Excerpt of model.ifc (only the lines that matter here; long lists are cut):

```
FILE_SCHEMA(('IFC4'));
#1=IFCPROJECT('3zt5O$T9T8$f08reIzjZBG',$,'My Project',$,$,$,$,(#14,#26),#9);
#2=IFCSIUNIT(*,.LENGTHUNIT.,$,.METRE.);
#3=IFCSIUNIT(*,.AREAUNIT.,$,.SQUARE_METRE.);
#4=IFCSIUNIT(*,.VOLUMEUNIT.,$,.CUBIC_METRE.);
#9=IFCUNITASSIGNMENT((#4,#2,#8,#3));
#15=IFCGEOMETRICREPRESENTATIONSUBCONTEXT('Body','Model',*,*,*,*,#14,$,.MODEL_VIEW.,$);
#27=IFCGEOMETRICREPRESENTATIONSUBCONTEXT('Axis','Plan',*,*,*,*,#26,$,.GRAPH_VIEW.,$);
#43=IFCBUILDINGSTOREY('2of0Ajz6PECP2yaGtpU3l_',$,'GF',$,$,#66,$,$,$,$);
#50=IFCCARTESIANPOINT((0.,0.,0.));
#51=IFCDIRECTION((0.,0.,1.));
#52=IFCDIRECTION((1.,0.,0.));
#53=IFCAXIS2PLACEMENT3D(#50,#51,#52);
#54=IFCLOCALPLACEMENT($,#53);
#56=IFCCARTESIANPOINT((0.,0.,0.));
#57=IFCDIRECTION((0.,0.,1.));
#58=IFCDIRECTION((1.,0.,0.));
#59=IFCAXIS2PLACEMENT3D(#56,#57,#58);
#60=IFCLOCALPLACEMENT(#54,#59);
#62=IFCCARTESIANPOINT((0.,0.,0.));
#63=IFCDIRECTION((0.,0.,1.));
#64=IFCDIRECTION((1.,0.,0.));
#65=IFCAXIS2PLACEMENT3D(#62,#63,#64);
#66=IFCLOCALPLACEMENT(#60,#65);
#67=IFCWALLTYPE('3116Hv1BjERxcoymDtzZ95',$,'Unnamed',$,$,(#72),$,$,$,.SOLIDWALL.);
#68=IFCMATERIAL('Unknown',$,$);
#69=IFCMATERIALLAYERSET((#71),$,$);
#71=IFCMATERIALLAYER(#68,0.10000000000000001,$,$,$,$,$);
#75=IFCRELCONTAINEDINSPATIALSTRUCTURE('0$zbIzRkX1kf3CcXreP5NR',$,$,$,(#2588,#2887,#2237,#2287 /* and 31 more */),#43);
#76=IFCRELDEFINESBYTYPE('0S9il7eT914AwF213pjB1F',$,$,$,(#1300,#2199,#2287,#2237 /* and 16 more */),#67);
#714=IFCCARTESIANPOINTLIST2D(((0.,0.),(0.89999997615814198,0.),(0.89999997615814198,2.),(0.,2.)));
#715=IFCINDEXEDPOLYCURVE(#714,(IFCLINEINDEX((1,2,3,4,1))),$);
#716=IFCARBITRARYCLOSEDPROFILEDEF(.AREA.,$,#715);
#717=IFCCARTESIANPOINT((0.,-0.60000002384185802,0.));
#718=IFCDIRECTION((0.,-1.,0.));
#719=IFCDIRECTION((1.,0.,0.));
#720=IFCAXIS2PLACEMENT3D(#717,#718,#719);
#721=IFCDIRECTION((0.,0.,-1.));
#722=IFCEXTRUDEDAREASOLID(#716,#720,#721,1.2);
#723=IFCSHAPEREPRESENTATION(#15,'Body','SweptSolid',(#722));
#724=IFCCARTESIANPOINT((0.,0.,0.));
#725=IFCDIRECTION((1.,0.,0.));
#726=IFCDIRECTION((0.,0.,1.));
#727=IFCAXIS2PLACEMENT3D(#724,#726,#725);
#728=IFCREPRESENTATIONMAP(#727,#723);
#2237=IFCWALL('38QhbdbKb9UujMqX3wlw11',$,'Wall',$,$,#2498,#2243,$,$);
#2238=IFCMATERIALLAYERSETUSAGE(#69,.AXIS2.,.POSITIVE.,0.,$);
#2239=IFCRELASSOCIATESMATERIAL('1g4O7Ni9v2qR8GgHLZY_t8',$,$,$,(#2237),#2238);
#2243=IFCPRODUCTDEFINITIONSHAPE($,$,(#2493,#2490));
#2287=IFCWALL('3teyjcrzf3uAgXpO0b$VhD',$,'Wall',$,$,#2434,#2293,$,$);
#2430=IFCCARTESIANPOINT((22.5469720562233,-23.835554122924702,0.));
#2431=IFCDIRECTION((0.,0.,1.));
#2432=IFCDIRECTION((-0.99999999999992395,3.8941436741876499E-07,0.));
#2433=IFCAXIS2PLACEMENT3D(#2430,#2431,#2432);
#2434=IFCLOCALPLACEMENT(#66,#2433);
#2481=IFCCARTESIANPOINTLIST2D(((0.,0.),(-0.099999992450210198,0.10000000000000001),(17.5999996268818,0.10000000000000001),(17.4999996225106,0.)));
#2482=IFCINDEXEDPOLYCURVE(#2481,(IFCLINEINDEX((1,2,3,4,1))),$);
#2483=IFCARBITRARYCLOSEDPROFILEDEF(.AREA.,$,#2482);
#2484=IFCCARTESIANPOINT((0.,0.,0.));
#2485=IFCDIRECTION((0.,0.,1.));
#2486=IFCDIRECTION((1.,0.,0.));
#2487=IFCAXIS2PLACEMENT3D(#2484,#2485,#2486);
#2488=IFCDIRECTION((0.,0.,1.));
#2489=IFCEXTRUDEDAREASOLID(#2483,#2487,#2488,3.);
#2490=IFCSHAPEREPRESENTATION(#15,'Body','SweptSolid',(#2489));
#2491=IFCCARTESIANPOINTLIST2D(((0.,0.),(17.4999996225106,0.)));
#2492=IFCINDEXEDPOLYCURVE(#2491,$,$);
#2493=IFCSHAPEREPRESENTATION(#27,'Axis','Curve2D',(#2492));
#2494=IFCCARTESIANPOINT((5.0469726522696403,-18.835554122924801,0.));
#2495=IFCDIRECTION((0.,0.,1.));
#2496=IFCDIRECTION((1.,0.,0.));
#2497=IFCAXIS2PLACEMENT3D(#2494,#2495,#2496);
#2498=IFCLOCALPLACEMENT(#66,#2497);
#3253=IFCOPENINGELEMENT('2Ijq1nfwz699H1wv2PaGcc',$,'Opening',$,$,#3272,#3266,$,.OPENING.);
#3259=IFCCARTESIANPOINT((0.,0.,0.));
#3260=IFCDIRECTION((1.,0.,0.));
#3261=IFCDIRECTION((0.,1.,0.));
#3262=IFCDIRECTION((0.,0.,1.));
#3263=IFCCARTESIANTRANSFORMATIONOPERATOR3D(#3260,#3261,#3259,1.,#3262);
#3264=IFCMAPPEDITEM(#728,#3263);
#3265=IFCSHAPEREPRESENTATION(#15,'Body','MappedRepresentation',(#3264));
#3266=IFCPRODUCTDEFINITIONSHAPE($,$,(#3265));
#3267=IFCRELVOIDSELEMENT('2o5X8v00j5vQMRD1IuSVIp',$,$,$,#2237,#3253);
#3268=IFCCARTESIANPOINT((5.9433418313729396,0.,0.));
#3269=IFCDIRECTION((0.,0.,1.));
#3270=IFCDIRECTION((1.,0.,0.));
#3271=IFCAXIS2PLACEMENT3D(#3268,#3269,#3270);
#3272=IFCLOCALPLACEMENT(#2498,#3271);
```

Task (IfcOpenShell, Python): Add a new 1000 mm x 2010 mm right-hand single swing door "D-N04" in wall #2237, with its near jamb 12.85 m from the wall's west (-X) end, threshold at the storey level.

```python
import numpy as np
import ifcopenshell
import ifcopenshell.api.feature
import ifcopenshell.api.geometry
import ifcopenshell.api.root
import ifcopenshell.api.spatial
import ifcopenshell.geom
import ifcopenshell.util.element
import ifcopenshell.util.placement
import ifcopenshell.util.representation
import ifcopenshell.util.shape
import ifcopenshell.util.unit

model = ifcopenshell.open("model.ifc")
unit_scale = ifcopenshell.util.unit.calculate_unit_scale(model)
settings = ifcopenshell.geom.settings()


def volume(element):
    """Net volume in cubic metres, openings subtracted."""
    shape = ifcopenshell.geom.create_shape(settings, element)
    return ifcopenshell.util.shape.get_volume(shape.geometry)


wall = model.by_id(2237)
storey = ifcopenshell.util.element.get_container(wall, ifc_class="IfcBuildingStorey")
context = ifcopenshell.util.representation.get_context(model, "Model", "Body", "MODEL_VIEW")
before = volume(wall)

width, height, from_end, sill = 1, 2.01, 12.85, 0.0  # metres

# The wall runs along its own X axis, and the end named is its -X end.
wall_shape = ifcopenshell.geom.create_shape(settings, wall)
x, y, z = ifcopenshell.util.shape.get_vertices(wall_shape.geometry).T
start = x.min() + from_end
face, thickness = float(y.min()), float(y.max() - y.min())
wall_matrix = ifcopenshell.util.placement.get_local_placement(wall.ObjectPlacement)
level = ifcopenshell.util.placement.get_local_placement(storey.ObjectPlacement)[2, 3]


def in_wall(x, y):
    """Placement at x, y metres in the wall's axes, at sill height."""
    matrix = wall_matrix.copy()
    matrix[:, 3] = wall_matrix @ np.array([x / unit_scale, y / unit_scale, 0.0, 1.0])
    matrix[2, 3] = level + sill / unit_scale
    return matrix


# Opening: a box that overshoots both wall faces by 50 mm.
opening = ifcopenshell.api.root.create_entity(model, ifc_class="IfcOpeningElement", predefined_type="OPENING")
box = ifcopenshell.api.geometry.add_wall_representation(
    model, context=context, length=width, height=height, thickness=thickness + 0.1
)
ifcopenshell.api.geometry.assign_representation(model, product=opening, representation=box)
ifcopenshell.api.geometry.edit_object_placement(model, product=opening, matrix=in_wall(start, face - 0.05), is_si=False)
ifcopenshell.api.feature.add_feature(model, feature=opening, element=wall)

door = ifcopenshell.api.root.create_entity(model, ifc_class="IfcDoor", name="D-N04", predefined_type="DOOR")
door.OverallWidth, door.OverallHeight = width / unit_scale, height / unit_scale
door.OperationType = "SINGLE_SWING_RIGHT"
body = ifcopenshell.api.geometry.add_door_representation(
    model,
    context=context,
    overall_width=door.OverallWidth,
    overall_height=door.OverallHeight,
    operation_type="SINGLE_SWING_RIGHT",
    lining_properties={"LiningDepth": thickness / unit_scale, "ThresholdDepth": thickness / unit_scale},
)
ifcopenshell.api.geometry.assign_representation(model, product=door, representation=body)
ifcopenshell.api.spatial.assign_container(model, products=[door], relating_structure=storey)
ifcopenshell.api.feature.add_filling(model, opening=opening, element=door)

# The lining spans the wall, so the door starts at the wall face.
ifcopenshell.api.geometry.edit_object_placement(model, product=door, matrix=in_wall(start, face), is_si=False)

after = volume(wall)

print(f"wall volume {before:.3f} -> {after:.3f} m3")

model.write("model_updated.ifc")
```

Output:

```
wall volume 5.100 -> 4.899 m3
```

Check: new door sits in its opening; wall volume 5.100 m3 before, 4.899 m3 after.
